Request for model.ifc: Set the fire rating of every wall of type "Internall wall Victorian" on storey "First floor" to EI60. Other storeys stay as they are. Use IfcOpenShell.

First a look at what the model holds.

```python
import ifcopenshell
import ifcopenshell.util.element

model = ifcopenshell.open("model.ifc")
print(model.schema)
storey = next(s for s in model.by_type("IfcBuildingStorey") if s.Name == "First floor")
walls = [e for e in ifcopenshell.util.element.get_decomposition(storey) if e.is_a("IfcWall")]
seen = {}
for e in walls:
    element_type = ifcopenshell.util.element.get_type(e)
    key = (element_type.Name if element_type != e and element_type else None, ifcopenshell.util.element.get_pset(e, "Pset_WallCommon", "FireRating"))
    seen[key] = seen.get(key, 0) + 1
for (name, value), count in sorted(seen.items(), key=str):
    print(count, "x", name, "|", value)
```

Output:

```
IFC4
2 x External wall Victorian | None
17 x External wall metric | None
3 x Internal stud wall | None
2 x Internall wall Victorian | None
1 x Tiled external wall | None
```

```python
import ifcopenshell
import ifcopenshell.api.pset
import ifcopenshell.util.element

model = ifcopenshell.open("model.ifc")

storey = next(s for s in model.by_type("IfcBuildingStorey") if s.Name == "First floor")
walls = [e for e in ifcopenshell.util.element.get_decomposition(storey) if e.is_a("IfcWall")]

count = 0
for e in walls:
    element_type = ifcopenshell.util.element.get_type(e)
    if element_type in (None, e) or element_type.Name != "Internall wall Victorian":
        continue
    # add_pset returns the element's existing set when there is one.
    pset = ifcopenshell.api.pset.add_pset(model, product=e, name="Pset_WallCommon")
    ifcopenshell.api.pset.edit_pset(model, pset=pset, properties={"FireRating": "EI60"})
    count += 1

print(count, "walls updated")

model.write("model_edited.ifc")
```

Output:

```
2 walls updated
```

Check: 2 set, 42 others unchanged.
